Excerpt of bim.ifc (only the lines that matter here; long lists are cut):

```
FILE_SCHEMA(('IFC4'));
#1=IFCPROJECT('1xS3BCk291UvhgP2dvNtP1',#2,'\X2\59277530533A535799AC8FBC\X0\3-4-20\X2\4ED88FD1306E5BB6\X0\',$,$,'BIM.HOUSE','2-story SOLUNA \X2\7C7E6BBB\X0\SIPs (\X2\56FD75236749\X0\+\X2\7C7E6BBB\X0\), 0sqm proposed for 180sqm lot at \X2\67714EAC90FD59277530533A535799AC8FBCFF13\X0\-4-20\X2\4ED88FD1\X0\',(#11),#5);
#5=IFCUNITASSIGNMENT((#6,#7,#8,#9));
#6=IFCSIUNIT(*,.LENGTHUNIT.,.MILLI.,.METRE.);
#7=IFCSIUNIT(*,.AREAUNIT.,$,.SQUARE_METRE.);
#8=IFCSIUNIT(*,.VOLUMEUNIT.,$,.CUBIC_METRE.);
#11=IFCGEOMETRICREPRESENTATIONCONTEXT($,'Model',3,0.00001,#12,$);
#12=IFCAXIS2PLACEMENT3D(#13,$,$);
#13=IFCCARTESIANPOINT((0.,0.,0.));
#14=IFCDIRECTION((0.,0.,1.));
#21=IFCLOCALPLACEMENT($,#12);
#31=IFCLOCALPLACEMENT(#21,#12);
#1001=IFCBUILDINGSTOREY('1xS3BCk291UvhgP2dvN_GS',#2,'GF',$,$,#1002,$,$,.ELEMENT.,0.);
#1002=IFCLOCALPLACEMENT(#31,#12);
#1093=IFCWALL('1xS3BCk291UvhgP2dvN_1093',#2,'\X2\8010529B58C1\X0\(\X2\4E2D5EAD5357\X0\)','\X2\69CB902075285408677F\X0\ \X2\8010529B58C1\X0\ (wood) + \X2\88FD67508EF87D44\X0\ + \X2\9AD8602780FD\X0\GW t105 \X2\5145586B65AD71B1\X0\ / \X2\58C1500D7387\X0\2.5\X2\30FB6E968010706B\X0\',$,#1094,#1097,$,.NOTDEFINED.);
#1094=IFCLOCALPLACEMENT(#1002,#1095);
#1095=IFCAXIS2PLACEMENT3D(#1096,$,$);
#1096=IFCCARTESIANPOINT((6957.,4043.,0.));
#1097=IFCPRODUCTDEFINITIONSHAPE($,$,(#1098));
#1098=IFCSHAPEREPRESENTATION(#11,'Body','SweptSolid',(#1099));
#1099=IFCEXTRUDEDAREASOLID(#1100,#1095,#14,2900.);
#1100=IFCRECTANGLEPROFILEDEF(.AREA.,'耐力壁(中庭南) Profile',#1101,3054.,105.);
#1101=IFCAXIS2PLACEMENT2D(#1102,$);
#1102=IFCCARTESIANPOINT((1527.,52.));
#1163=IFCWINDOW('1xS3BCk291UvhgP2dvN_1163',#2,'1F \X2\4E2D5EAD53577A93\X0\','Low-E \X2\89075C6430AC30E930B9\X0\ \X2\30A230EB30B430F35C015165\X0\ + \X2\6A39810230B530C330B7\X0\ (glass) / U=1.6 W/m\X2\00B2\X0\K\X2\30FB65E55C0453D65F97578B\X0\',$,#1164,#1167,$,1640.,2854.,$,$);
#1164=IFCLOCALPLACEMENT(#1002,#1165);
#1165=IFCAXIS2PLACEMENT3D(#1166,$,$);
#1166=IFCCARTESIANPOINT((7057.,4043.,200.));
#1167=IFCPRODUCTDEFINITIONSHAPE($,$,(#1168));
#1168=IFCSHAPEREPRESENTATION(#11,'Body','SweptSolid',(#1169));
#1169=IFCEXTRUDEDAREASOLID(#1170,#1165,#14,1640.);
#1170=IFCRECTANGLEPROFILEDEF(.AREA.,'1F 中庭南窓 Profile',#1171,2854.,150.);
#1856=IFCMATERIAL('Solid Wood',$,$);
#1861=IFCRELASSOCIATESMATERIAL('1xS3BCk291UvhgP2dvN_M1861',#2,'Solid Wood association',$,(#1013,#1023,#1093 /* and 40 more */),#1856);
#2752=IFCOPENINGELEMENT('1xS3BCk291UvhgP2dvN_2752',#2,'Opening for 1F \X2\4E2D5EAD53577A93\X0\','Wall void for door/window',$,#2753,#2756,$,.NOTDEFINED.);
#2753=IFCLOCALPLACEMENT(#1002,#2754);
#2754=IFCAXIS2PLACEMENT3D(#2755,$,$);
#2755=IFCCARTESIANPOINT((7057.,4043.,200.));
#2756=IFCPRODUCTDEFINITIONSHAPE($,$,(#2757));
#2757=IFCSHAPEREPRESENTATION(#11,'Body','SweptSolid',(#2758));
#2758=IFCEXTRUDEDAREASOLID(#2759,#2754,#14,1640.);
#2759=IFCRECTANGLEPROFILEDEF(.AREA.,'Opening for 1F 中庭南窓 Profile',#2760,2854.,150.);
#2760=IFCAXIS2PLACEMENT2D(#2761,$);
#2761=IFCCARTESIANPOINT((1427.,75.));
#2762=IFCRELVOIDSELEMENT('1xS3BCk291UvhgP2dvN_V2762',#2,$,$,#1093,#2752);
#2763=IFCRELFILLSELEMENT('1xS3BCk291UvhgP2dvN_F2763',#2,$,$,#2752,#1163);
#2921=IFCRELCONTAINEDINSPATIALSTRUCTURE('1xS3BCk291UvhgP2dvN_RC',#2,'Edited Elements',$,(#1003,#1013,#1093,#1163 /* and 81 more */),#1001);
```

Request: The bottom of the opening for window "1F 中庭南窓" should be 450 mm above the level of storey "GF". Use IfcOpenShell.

```python
import numpy as np
import ifcopenshell
import ifcopenshell.api.geometry
import ifcopenshell.geom
import ifcopenshell.util.element
import ifcopenshell.util.placement
import ifcopenshell.util.shape
import ifcopenshell.util.unit

model = ifcopenshell.open("bim.ifc")
unit_scale = ifcopenshell.util.unit.calculate_unit_scale(model)

window = model.by_guid("1xS3BCk291UvhgP2dvN_1163")
opening = window.FillsVoids[0].RelatingOpeningElement
storey = ifcopenshell.util.element.get_container(window, ifc_class="IfcBuildingStorey")
level = ifcopenshell.util.placement.get_local_placement(storey.ObjectPlacement)[2, 3]

# The opening's origin need not be at the sill, so measure its lowest point.
shape = ifcopenshell.geom.create_shape(ifcopenshell.geom.settings(), opening)
bottom = ifcopenshell.util.shape.get_shape_bottom_elevation(shape, shape.geometry) / unit_scale
dz = level + 450.0 - bottom

shift = np.array([0.0, 0.0, dz])
# The window is not placed relative to its opening, so move both.
for product in (opening, window):
    matrix = ifcopenshell.util.placement.get_local_placement(product.ObjectPlacement)
    matrix[:3, 3] += shift
    ifcopenshell.api.geometry.edit_object_placement(model, product=product, matrix=matrix, is_si=False)

print(f"moved by {dz * unit_scale:+.3f} m")

model.write("bim_updated.ifc")
```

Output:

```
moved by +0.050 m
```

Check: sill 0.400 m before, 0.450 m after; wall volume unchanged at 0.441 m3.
